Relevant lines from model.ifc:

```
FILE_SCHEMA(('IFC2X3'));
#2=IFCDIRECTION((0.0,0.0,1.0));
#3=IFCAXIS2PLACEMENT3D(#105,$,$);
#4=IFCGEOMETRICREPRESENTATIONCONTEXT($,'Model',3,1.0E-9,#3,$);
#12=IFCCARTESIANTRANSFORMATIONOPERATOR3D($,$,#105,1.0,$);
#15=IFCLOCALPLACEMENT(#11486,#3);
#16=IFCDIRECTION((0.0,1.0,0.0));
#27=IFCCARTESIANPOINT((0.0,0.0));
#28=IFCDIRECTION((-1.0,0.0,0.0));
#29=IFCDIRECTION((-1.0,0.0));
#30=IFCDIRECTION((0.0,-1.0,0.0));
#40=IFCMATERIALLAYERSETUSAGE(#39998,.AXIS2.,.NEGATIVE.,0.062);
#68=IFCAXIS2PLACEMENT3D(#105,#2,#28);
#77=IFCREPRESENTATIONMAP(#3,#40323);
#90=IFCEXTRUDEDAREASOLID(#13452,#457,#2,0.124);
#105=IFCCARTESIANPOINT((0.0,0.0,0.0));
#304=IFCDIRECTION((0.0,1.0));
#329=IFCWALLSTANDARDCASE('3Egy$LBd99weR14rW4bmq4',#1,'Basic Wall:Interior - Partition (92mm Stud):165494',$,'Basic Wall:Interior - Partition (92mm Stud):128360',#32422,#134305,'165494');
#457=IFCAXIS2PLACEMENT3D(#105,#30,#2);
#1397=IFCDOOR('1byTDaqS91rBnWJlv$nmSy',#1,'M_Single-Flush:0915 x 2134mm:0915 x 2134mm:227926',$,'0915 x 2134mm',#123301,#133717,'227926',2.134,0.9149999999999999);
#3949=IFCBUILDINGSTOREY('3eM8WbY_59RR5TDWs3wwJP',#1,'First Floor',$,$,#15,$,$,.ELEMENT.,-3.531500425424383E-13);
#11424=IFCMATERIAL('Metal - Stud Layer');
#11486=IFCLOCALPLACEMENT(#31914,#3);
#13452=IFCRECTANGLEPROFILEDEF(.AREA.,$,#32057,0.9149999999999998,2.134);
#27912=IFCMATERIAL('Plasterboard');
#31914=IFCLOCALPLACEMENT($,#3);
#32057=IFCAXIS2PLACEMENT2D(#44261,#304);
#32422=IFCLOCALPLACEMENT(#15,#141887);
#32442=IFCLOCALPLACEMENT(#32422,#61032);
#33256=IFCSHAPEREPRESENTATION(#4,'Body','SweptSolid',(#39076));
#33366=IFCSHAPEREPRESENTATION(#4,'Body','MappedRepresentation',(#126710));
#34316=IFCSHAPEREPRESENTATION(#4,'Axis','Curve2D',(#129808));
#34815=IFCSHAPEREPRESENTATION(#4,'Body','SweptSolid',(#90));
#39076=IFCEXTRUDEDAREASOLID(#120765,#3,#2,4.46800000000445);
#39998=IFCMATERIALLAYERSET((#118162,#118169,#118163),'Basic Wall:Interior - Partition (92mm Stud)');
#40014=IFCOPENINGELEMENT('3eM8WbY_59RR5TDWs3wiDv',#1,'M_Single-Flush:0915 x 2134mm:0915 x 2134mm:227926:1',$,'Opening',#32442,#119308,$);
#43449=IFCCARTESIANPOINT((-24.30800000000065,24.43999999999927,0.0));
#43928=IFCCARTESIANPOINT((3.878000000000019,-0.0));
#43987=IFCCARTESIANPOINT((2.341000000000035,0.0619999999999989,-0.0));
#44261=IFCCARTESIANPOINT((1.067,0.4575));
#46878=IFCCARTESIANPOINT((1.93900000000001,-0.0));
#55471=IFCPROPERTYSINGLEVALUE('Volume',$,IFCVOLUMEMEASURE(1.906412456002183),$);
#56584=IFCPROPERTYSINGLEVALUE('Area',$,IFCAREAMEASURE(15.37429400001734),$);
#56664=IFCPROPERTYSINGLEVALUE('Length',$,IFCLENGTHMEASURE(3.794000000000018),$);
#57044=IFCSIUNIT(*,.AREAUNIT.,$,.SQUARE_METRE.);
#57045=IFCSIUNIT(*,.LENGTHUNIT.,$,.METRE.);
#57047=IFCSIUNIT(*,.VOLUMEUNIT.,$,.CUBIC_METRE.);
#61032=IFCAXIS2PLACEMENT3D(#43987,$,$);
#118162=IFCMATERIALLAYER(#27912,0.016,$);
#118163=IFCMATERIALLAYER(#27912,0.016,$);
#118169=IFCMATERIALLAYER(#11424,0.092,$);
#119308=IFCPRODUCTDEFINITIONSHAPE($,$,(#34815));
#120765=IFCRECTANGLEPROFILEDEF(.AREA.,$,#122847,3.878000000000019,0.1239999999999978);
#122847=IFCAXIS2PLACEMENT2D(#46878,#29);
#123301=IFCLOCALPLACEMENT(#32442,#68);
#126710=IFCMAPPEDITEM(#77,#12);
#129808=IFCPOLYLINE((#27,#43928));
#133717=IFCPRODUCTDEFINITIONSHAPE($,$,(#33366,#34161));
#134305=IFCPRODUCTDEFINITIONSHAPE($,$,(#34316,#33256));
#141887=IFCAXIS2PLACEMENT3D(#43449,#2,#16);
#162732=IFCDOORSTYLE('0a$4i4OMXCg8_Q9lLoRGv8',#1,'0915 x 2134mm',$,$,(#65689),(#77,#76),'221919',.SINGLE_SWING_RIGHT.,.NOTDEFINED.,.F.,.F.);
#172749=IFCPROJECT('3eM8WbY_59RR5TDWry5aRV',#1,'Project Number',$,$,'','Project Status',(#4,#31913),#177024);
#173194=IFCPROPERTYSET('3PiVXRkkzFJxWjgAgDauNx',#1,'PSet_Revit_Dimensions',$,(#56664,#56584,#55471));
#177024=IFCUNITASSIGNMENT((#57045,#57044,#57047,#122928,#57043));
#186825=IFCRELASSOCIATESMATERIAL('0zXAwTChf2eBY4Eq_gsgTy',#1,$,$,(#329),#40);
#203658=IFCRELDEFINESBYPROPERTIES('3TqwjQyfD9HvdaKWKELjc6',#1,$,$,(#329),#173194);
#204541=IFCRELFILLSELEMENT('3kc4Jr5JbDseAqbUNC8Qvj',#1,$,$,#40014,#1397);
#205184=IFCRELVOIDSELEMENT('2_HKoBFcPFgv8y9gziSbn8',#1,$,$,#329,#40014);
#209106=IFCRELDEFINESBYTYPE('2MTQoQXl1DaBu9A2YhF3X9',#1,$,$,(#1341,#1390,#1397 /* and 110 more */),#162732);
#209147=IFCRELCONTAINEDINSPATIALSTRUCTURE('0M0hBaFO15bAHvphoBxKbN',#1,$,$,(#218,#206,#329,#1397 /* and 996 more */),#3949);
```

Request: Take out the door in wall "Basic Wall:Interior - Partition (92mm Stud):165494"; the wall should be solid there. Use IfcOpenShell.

```python
import ifcopenshell
import ifcopenshell.api.feature
import ifcopenshell.api.pset
import ifcopenshell.api.root
import ifcopenshell.geom
import ifcopenshell.util.element
import ifcopenshell.util.shape
import ifcopenshell.util.unit

model = ifcopenshell.open("model.ifc")
area_scale = ifcopenshell.util.unit.calculate_unit_scale(model, "AREAUNIT")
volume_scale = ifcopenshell.util.unit.calculate_unit_scale(model, "VOLUMEUNIT")
settings = ifcopenshell.geom.settings()


def volume(element):
    """Net volume in cubic metres, openings subtracted."""
    shape = ifcopenshell.geom.create_shape(settings, element)
    return ifcopenshell.util.shape.get_volume(shape.geometry)


door = model.by_guid("1byTDaqS91rBnWJlv$nmSy")
opening = door.FillsVoids[0].RelatingOpeningElement
wall = opening.VoidsElements[0].RelatingBuildingElement
before = volume(wall)

ifcopenshell.api.root.remove_product(model, product=door)
ifcopenshell.api.feature.remove_feature(model, feature=opening)

after = volume(wall)
thickness = 0.124  # wall thickness in metres

# Update the wall's stored quantities.
pset = model.by_id(ifcopenshell.util.element.get_pset(wall, "PSet_Revit_Dimensions", should_inherit=False)["id"])
ifcopenshell.api.pset.edit_pset(model, pset=pset, properties={
    "Area": model.create_entity("IfcAreaMeasure", after / thickness / area_scale),
    "Volume": model.create_entity("IfcVolumeMeasure", after / volume_scale),
})

print(f"wall volume {before:.3f} -> {after:.3f} m3")

model.write("model-out.ifc")
```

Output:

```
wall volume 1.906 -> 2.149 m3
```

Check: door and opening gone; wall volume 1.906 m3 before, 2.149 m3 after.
